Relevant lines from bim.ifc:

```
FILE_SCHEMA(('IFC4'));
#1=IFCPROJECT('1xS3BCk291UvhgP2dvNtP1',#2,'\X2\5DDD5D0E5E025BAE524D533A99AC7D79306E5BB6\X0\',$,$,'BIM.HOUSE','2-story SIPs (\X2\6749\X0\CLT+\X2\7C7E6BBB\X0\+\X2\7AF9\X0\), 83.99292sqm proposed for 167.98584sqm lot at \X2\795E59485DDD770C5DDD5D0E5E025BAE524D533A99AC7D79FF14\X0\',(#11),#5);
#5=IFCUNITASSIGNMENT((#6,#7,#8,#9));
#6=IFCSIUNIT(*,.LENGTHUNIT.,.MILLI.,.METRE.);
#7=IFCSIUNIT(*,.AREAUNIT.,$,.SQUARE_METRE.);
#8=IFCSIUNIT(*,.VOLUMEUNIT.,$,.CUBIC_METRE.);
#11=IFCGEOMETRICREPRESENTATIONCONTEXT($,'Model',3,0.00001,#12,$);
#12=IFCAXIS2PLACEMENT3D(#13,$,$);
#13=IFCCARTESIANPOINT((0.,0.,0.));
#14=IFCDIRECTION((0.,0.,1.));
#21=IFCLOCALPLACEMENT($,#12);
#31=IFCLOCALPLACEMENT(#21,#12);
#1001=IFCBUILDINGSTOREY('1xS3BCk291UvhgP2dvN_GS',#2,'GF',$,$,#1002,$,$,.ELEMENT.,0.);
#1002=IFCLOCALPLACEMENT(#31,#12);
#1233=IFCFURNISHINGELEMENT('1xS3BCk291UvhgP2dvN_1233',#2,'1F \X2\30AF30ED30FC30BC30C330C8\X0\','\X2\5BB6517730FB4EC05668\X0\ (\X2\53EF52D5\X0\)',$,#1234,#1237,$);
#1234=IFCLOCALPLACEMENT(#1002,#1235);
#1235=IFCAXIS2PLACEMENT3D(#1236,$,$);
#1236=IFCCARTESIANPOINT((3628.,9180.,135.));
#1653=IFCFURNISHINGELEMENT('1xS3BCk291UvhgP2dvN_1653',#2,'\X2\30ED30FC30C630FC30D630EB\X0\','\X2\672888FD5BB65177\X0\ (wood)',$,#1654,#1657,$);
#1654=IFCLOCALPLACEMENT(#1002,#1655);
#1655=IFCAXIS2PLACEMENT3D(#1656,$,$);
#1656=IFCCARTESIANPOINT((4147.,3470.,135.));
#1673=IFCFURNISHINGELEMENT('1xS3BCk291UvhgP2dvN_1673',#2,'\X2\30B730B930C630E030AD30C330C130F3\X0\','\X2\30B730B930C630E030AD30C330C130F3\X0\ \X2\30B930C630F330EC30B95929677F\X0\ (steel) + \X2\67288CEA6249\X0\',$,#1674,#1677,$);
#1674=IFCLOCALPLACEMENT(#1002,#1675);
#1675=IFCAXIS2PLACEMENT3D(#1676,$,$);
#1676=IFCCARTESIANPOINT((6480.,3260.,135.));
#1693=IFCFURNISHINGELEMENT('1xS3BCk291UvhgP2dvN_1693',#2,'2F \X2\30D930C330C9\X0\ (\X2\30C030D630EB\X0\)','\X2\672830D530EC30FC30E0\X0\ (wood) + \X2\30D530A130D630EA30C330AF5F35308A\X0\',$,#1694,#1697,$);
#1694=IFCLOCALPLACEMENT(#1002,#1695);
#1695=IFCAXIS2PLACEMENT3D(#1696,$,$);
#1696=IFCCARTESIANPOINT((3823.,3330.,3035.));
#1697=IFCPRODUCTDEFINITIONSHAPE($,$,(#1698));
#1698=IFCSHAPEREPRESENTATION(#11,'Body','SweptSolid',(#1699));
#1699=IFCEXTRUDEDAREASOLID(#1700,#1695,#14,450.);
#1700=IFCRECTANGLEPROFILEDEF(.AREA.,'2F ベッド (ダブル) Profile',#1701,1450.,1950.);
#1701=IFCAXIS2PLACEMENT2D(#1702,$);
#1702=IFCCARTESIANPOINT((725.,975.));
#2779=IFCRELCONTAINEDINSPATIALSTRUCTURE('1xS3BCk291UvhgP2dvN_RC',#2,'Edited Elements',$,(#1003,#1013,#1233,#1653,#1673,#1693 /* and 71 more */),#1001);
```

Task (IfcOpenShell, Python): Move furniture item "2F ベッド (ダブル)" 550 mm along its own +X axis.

```python
import ifcopenshell
import ifcopenshell.api.geometry
import ifcopenshell.util.placement

model = ifcopenshell.open("bim.ifc")

item = model.by_guid("1xS3BCk291UvhgP2dvN_1693")
matrix = ifcopenshell.util.placement.get_local_placement(item.ObjectPlacement)
matrix[:3, 3] += matrix[:3, 0] * 550.0
ifcopenshell.api.geometry.edit_object_placement(model, product=item, matrix=matrix, is_si=False)

print(ifcopenshell.util.placement.get_local_placement(item.ObjectPlacement).round(3) + 0.0)

model.write("bim_updated.ifc")
```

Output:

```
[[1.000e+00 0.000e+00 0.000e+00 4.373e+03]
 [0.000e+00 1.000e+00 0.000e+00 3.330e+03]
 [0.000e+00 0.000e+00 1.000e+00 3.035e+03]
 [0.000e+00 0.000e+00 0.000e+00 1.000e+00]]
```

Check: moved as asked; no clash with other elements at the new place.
